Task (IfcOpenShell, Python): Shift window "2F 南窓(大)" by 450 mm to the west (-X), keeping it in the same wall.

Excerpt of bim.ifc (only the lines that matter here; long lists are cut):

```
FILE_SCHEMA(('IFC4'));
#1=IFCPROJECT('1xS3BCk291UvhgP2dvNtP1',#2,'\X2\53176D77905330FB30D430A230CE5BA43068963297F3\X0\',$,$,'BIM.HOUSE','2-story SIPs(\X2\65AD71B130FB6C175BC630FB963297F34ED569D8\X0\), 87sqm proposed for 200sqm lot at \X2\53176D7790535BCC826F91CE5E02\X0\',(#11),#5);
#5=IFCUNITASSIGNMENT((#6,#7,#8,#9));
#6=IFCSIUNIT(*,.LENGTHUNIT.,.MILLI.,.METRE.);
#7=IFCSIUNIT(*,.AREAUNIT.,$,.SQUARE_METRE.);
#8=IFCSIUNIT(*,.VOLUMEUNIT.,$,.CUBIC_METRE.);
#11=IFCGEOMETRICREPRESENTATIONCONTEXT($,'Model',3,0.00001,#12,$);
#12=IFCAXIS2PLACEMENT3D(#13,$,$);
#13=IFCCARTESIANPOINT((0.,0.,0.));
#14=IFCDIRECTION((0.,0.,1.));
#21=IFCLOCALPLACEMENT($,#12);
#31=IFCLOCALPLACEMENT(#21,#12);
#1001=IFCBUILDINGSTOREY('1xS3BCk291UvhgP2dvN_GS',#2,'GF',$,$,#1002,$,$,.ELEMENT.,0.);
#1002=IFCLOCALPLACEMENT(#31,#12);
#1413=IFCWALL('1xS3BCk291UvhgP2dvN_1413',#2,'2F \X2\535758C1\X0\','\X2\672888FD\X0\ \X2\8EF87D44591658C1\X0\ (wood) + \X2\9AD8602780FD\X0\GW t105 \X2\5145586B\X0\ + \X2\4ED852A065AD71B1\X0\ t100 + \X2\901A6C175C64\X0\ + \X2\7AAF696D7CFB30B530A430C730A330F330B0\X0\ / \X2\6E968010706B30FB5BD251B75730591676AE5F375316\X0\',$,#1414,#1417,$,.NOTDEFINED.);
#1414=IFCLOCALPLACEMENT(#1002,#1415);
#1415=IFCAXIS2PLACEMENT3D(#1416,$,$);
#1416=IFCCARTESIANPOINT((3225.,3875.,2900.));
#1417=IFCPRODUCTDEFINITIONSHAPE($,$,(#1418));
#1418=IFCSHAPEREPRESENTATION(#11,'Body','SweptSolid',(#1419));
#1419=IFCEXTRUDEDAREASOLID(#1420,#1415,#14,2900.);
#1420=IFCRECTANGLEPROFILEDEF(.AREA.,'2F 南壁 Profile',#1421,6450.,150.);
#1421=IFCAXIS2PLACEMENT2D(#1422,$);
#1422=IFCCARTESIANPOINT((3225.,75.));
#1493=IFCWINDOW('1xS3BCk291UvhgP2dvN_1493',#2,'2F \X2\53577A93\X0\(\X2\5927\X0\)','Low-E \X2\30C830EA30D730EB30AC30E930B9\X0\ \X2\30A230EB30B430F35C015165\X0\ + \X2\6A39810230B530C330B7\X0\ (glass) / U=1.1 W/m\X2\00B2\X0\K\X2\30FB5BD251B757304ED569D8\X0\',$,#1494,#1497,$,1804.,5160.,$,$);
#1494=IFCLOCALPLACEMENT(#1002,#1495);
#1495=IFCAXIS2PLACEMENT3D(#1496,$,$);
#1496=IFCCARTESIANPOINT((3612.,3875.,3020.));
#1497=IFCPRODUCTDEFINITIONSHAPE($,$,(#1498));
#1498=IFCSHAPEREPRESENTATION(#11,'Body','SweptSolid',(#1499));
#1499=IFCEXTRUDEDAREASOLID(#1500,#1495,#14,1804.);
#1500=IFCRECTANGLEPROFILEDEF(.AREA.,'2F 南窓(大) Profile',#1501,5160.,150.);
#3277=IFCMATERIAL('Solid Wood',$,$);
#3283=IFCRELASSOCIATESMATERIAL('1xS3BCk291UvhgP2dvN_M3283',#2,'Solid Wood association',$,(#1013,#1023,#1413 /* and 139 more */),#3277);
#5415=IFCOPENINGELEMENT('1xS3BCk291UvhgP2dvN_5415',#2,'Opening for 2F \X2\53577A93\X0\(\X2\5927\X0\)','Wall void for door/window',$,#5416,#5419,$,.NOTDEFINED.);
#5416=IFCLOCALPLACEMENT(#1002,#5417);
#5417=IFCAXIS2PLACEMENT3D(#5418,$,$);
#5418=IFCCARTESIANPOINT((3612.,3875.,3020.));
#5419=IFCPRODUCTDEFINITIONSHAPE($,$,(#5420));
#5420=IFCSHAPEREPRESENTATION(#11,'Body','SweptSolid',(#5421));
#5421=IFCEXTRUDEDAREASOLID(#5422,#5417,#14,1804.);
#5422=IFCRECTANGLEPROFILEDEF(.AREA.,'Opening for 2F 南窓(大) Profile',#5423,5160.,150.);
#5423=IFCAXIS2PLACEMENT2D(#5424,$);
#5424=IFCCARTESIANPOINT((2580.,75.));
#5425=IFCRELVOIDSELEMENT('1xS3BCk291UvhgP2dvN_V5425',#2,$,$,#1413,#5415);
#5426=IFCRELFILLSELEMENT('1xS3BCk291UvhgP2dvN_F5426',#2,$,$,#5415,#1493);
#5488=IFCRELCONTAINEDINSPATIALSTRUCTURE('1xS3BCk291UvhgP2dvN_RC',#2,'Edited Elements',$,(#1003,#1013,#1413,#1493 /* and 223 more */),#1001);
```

```python
import ifcopenshell
import ifcopenshell.api.geometry
import ifcopenshell.util.placement
import ifcopenshell.util.unit

model = ifcopenshell.open("bim.ifc")
unit_scale = ifcopenshell.util.unit.calculate_unit_scale(model)

window = model.by_id(1493)
opening = window.FillsVoids[0].RelatingOpeningElement
wall = opening.VoidsElements[0].RelatingBuildingElement

wall_matrix = ifcopenshell.util.placement.get_local_placement(wall.ObjectPlacement)
shift = wall_matrix[:3, 0] * -0.45 / unit_scale
before = ifcopenshell.util.placement.get_local_placement(window.ObjectPlacement)[:3, 3].copy()

# The window is not placed relative to its opening, so move both.
for product in (opening, window):
    matrix = ifcopenshell.util.placement.get_local_placement(product.ObjectPlacement)
    matrix[:3, 3] += shift
    ifcopenshell.api.geometry.edit_object_placement(model, product=product, matrix=matrix, is_si=False)

after = ifcopenshell.util.placement.get_local_placement(window.ObjectPlacement)[:3, 3]
print("window moved by", (after - before).round(3) + 0.0)

model.write("bim_updated.ifc")
```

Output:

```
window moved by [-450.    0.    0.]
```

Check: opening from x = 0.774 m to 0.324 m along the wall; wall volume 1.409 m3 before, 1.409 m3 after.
